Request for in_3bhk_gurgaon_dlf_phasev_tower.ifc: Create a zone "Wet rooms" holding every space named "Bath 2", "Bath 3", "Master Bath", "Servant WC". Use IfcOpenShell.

First a look at what the model holds.

```python
import ifcopenshell

model = ifcopenshell.open("in_3bhk_gurgaon_dlf_phasev_tower.ifc")
print(model.schema)
seen = {}
for space in model.by_type("IfcSpace"):
    seen[space.LongName] = seen.get(space.LongName, 0) + 1
for name, count in sorted(seen.items(), key=str):
    print(count, "x", name)
print("zones:", [z.Name for z in model.by_type("IfcZone")][:20])
```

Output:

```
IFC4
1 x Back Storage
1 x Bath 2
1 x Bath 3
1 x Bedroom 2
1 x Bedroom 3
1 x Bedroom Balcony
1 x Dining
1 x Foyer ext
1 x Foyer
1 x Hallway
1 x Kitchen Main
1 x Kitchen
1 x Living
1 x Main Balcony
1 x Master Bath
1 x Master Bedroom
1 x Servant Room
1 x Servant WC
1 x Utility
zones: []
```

```python
import ifcopenshell
import ifcopenshell.api.group
import ifcopenshell.api.root

model = ifcopenshell.open("in_3bhk_gurgaon_dlf_phasev_tower.ifc")

names = {"Bath 2", "Bath 3", "Master Bath", "Servant WC"}
spaces = [s for s in model.by_type("IfcSpace") if s.LongName in names]

zone = ifcopenshell.api.root.create_entity(model, ifc_class="IfcZone", name="Wet rooms")
ifcopenshell.api.group.assign_group(model, products=spaces, group=zone)
print(len(spaces), "spaces in", zone.Name)

model.write("in_3bhk_gurgaon_dlf_phasev_tower-out.ifc")
```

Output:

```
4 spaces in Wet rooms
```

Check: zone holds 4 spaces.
